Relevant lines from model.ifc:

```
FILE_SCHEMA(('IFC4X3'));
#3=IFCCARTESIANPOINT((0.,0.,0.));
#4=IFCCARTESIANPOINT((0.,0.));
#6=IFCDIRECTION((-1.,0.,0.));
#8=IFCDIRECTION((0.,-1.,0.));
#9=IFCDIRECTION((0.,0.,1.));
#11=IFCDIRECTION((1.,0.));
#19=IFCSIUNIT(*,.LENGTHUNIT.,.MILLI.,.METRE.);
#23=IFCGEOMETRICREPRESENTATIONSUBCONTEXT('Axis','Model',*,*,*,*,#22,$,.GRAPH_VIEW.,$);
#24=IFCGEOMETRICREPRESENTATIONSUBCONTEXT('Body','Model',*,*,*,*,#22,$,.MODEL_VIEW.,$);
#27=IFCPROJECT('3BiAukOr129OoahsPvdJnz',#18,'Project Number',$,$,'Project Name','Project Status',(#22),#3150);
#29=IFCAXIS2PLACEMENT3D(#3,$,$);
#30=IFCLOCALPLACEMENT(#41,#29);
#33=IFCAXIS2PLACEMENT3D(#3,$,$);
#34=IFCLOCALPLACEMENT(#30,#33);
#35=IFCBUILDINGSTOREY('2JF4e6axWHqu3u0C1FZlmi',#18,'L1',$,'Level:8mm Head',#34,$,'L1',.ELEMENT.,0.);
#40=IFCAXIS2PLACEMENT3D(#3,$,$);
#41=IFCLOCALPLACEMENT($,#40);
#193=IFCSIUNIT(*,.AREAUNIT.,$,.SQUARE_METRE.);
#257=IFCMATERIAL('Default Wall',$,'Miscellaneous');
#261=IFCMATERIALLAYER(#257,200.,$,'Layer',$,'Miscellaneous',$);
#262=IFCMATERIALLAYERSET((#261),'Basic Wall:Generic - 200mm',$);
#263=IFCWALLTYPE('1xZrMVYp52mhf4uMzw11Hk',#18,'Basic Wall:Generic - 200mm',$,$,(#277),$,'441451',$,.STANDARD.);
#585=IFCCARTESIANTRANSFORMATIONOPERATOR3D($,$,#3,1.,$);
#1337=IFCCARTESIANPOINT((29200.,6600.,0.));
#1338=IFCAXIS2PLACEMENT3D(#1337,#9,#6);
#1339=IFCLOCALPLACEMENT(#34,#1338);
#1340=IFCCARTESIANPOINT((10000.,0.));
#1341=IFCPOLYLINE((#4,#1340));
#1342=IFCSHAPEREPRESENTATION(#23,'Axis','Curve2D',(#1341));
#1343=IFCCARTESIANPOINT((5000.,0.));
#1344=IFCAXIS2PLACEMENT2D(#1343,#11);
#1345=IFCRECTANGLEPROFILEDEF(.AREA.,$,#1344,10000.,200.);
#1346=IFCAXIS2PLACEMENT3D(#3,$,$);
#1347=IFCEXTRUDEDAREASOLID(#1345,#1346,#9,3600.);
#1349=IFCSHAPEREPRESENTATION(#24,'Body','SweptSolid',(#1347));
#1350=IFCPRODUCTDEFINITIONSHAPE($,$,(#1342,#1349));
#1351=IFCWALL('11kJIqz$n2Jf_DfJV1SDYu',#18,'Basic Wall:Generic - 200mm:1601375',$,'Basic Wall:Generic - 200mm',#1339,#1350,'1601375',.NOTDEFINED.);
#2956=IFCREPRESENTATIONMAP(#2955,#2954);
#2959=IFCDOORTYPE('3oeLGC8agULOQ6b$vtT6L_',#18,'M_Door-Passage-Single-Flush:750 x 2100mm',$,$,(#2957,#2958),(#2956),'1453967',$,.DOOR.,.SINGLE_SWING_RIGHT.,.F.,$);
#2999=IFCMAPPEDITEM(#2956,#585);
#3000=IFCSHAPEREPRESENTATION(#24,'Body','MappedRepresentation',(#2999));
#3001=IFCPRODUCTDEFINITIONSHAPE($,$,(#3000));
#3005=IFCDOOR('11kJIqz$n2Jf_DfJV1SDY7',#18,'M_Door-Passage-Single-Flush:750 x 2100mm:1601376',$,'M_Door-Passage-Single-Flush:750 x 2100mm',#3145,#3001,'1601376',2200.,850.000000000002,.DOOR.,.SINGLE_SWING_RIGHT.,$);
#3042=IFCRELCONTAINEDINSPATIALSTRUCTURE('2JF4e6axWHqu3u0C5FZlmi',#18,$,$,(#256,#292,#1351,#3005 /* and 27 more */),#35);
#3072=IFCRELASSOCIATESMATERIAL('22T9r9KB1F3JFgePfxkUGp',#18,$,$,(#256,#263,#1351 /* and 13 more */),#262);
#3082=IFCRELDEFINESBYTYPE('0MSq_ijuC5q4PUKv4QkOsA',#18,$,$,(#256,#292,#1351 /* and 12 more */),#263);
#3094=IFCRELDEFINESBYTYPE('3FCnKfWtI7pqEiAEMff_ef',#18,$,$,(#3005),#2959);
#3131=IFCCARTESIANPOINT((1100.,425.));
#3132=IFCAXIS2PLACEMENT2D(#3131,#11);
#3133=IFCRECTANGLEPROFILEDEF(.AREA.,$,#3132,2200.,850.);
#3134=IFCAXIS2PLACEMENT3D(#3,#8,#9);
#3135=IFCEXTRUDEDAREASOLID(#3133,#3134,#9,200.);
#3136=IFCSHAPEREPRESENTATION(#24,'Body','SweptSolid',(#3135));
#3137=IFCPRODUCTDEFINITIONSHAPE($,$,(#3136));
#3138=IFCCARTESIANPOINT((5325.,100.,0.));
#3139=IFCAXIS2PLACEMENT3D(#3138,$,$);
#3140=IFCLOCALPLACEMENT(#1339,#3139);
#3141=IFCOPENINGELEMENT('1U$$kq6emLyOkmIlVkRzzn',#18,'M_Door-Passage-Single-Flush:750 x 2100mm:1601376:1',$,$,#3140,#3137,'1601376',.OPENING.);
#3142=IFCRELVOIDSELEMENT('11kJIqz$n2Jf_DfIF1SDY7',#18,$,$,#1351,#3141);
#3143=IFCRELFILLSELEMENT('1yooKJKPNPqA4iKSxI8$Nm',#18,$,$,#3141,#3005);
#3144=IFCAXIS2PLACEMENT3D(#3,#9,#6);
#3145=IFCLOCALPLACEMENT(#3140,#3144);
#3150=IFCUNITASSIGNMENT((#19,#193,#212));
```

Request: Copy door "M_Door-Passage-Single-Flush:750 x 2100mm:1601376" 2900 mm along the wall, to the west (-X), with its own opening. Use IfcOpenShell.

```python
import ifcopenshell
import ifcopenshell.api.feature
import ifcopenshell.api.geometry
import ifcopenshell.api.root
import ifcopenshell.geom
import ifcopenshell.util.element
import ifcopenshell.util.placement
import ifcopenshell.util.shape

model = ifcopenshell.open("model.ifc")
settings = ifcopenshell.geom.settings()


def volume(element):
    """Net volume in cubic metres, openings subtracted."""
    shape = ifcopenshell.geom.create_shape(settings, element)
    return ifcopenshell.util.shape.get_volume(shape.geometry)


def reuse_history(source, copy):
    """copy_class also copies each property set's owner history, people and application; keep the originals."""
    for rel in copy.IsDefinedBy:
        if rel.is_a("IfcRelDefinesByProperties") and (history := rel.RelatingPropertyDefinition.OwnerHistory):
            rel.RelatingPropertyDefinition.OwnerHistory = source.OwnerHistory
            ifcopenshell.util.element.remove_deep2(model, history)


door = model.by_guid("11kJIqz$n2Jf_DfJV1SDY7")
opening = door.FillsVoids[0].RelatingOpeningElement
wall = opening.VoidsElements[0].RelatingBuildingElement
before = volume(wall)
shift = ifcopenshell.util.placement.get_local_placement(wall.ObjectPlacement)[:3, 0] * 2900.0

# copy_class copies the void relationship, type, container and properties, but no geometry.
new_opening = ifcopenshell.api.root.copy_class(model, product=opening)
new_opening.Representation = ifcopenshell.util.element.copy_deep(
    model, opening.Representation, exclude=["IfcGeometricRepresentationContext", "IfcRepresentationMap"]
)
new_opening.Name = "M_Door-Passage-Single-Flush:750 x 2100mm"
new_opening.Tag = None
new_door = ifcopenshell.api.root.copy_class(model, product=door)
new_door.Representation = ifcopenshell.util.element.copy_deep(
    model, door.Representation, exclude=["IfcGeometricRepresentationContext", "IfcRepresentationMap"]
)
new_door.Name = "M_Door-Passage-Single-Flush:750 x 2100mm"
new_door.Tag = None
reuse_history(door, new_door)
ifcopenshell.api.feature.add_filling(model, opening=new_opening, element=new_door)

for old, new in ((opening, new_opening), (door, new_door)):
    matrix = ifcopenshell.util.placement.get_local_placement(old.ObjectPlacement)
    matrix[:3, 3] += shift
    ifcopenshell.api.geometry.edit_object_placement(model, product=new, matrix=matrix, is_si=False)

after = volume(wall)

print(f"wall volume {before:.3f} -> {after:.3f} m3")

model.write("model-out.ifc")
```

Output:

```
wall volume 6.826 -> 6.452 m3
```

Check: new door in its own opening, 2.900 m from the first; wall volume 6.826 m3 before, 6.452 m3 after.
